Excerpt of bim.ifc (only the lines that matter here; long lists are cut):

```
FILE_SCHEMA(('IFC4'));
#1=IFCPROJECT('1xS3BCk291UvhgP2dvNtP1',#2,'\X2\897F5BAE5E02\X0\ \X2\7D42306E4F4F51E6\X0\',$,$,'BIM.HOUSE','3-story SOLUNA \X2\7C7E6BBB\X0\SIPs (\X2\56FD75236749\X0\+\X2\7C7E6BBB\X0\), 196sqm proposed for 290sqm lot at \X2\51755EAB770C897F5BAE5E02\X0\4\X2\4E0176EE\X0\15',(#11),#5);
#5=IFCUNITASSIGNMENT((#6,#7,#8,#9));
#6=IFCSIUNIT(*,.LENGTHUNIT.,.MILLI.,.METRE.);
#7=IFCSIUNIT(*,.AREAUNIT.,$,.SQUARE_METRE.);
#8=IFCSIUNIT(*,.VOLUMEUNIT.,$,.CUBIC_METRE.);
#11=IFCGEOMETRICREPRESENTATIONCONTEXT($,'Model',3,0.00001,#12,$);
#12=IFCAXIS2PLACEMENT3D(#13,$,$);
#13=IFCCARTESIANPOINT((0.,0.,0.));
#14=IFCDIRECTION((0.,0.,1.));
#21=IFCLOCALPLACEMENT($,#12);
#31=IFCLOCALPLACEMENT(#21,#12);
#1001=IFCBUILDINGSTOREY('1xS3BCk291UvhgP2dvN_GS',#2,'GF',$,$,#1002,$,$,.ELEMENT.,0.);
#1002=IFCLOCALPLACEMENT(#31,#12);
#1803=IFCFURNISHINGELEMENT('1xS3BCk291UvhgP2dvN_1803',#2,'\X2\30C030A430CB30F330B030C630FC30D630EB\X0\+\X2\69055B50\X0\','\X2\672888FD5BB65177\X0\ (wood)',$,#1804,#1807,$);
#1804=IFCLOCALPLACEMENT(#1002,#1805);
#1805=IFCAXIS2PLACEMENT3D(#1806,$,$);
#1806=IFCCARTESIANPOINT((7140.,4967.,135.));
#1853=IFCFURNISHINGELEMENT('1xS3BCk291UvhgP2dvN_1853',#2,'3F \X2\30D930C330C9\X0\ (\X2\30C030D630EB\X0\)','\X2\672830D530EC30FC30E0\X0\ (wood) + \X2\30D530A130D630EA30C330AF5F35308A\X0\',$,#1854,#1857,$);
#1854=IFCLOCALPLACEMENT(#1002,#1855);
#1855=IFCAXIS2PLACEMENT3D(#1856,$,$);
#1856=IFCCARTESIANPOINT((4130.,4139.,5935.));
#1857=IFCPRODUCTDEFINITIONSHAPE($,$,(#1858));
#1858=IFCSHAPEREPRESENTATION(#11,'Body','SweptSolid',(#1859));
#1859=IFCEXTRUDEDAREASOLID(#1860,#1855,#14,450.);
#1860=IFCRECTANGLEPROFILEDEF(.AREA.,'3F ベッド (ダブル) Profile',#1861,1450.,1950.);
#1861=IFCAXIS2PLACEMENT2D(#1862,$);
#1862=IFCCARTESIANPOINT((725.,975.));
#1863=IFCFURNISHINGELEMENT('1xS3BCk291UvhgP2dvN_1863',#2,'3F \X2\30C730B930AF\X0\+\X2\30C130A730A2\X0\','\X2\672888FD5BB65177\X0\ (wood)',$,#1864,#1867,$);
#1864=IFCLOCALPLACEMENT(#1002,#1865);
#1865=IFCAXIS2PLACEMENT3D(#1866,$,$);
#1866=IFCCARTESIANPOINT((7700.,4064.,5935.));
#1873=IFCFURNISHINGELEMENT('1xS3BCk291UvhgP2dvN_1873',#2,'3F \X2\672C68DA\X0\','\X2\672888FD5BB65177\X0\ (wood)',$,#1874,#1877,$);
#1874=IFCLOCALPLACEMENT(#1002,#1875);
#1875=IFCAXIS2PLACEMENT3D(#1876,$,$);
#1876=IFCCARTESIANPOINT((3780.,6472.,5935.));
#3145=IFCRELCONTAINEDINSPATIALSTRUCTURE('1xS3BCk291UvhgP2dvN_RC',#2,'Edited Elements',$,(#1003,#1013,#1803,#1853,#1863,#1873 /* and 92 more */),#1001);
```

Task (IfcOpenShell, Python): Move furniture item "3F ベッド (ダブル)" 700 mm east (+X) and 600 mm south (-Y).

```python
import ifcopenshell
import ifcopenshell.api.geometry
import ifcopenshell.util.placement
import ifcopenshell.util.unit

model = ifcopenshell.open("bim.ifc")
unit_scale = ifcopenshell.util.unit.calculate_unit_scale(model)

item = model.by_id(1853)
matrix = ifcopenshell.util.placement.get_local_placement(item.ObjectPlacement)
matrix[0, 3] += 0.7 / unit_scale
matrix[1, 3] -= 0.6 / unit_scale
ifcopenshell.api.geometry.edit_object_placement(model, product=item, matrix=matrix, is_si=False)

print(ifcopenshell.util.placement.get_local_placement(item.ObjectPlacement).round(3) + 0.0)

model.write("bim_rev.ifc")
```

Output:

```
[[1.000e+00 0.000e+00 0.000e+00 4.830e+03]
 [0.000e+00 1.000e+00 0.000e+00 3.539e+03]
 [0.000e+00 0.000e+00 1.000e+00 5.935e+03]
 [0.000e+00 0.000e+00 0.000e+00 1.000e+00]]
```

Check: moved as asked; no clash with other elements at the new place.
